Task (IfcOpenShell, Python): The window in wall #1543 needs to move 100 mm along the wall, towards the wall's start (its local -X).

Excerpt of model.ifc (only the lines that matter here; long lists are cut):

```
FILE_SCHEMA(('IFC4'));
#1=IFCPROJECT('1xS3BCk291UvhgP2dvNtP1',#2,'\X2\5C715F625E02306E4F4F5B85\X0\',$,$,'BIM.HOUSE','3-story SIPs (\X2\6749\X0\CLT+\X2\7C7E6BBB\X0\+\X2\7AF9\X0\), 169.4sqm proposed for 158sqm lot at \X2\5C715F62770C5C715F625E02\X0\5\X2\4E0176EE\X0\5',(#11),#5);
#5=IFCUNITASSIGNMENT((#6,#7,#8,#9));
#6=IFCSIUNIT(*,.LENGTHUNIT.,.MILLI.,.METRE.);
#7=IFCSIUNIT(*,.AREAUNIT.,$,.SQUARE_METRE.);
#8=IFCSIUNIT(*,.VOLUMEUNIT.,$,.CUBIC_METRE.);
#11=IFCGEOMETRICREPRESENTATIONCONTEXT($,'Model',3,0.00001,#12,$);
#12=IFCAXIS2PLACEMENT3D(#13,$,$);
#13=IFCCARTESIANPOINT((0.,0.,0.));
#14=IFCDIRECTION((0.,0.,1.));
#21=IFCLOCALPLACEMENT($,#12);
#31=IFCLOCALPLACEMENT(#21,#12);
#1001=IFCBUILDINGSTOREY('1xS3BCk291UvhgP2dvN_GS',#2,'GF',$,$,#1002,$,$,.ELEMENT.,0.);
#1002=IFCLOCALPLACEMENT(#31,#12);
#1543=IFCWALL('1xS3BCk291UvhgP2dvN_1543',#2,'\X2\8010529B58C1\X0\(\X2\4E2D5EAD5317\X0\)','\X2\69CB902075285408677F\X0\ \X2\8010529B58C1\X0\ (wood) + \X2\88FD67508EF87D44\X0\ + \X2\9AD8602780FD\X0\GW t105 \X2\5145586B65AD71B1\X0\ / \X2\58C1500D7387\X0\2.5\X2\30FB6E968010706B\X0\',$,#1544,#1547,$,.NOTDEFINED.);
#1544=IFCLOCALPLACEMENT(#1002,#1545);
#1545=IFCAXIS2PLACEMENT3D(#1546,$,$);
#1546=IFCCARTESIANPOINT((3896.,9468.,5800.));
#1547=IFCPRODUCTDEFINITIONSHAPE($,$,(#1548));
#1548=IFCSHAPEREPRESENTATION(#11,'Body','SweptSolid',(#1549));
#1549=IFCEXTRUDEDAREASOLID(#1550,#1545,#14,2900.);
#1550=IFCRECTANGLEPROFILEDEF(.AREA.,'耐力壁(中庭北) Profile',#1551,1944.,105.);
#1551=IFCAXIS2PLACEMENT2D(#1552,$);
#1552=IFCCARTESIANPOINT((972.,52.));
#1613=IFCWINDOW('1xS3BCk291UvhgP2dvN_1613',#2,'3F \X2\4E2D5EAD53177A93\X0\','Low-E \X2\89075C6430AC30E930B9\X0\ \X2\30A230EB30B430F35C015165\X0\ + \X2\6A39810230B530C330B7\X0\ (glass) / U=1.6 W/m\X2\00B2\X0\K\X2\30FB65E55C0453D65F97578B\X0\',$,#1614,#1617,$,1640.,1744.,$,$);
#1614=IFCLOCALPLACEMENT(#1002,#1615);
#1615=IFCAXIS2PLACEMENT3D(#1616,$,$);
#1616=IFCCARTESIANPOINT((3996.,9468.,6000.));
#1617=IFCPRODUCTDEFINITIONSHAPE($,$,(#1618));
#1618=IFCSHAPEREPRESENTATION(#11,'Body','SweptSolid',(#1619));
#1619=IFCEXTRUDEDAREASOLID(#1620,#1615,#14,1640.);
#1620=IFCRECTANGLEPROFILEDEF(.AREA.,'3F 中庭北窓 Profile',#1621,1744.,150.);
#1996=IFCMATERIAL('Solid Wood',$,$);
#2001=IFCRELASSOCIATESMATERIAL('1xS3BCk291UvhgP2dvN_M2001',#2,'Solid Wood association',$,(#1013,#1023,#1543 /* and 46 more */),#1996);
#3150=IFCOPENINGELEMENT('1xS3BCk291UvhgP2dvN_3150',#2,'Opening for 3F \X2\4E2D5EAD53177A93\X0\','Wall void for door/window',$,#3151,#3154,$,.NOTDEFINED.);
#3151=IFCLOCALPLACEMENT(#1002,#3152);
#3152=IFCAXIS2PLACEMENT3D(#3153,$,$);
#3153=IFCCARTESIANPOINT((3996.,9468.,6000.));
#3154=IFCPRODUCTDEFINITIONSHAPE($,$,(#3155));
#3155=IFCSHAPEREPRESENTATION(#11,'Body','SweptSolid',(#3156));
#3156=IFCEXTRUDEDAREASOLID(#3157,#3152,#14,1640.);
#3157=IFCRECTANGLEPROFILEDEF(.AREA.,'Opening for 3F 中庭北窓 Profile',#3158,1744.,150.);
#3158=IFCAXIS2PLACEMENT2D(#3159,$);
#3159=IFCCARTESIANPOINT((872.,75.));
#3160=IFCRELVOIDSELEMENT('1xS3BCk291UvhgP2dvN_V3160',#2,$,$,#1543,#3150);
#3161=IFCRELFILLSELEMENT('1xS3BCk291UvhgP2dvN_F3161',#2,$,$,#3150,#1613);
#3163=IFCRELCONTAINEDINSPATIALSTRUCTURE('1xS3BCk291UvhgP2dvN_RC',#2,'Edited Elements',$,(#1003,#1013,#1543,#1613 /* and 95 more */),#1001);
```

```python
import ifcopenshell
import ifcopenshell.api.geometry
import ifcopenshell.util.placement
import ifcopenshell.util.unit

model = ifcopenshell.open("model.ifc")
unit_scale = ifcopenshell.util.unit.calculate_unit_scale(model)

window = model.by_guid("1xS3BCk291UvhgP2dvN_1613")
opening = window.FillsVoids[0].RelatingOpeningElement
wall = opening.VoidsElements[0].RelatingBuildingElement

wall_matrix = ifcopenshell.util.placement.get_local_placement(wall.ObjectPlacement)
shift = wall_matrix[:3, 0] * -0.1 / unit_scale
before = ifcopenshell.util.placement.get_local_placement(window.ObjectPlacement)[:3, 3].copy()

# The window is not placed relative to its opening, so move both.
for product in (opening, window):
    matrix = ifcopenshell.util.placement.get_local_placement(product.ObjectPlacement)
    matrix[:3, 3] += shift
    ifcopenshell.api.geometry.edit_object_placement(model, product=product, matrix=matrix, is_si=False)

after = ifcopenshell.util.placement.get_local_placement(window.ObjectPlacement)[:3, 3]
print("window moved by", (after - before).round(3) + 0.0)

model.write("model_edited.ifc")
```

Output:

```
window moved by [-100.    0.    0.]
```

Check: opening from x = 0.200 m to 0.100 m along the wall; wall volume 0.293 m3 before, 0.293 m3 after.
